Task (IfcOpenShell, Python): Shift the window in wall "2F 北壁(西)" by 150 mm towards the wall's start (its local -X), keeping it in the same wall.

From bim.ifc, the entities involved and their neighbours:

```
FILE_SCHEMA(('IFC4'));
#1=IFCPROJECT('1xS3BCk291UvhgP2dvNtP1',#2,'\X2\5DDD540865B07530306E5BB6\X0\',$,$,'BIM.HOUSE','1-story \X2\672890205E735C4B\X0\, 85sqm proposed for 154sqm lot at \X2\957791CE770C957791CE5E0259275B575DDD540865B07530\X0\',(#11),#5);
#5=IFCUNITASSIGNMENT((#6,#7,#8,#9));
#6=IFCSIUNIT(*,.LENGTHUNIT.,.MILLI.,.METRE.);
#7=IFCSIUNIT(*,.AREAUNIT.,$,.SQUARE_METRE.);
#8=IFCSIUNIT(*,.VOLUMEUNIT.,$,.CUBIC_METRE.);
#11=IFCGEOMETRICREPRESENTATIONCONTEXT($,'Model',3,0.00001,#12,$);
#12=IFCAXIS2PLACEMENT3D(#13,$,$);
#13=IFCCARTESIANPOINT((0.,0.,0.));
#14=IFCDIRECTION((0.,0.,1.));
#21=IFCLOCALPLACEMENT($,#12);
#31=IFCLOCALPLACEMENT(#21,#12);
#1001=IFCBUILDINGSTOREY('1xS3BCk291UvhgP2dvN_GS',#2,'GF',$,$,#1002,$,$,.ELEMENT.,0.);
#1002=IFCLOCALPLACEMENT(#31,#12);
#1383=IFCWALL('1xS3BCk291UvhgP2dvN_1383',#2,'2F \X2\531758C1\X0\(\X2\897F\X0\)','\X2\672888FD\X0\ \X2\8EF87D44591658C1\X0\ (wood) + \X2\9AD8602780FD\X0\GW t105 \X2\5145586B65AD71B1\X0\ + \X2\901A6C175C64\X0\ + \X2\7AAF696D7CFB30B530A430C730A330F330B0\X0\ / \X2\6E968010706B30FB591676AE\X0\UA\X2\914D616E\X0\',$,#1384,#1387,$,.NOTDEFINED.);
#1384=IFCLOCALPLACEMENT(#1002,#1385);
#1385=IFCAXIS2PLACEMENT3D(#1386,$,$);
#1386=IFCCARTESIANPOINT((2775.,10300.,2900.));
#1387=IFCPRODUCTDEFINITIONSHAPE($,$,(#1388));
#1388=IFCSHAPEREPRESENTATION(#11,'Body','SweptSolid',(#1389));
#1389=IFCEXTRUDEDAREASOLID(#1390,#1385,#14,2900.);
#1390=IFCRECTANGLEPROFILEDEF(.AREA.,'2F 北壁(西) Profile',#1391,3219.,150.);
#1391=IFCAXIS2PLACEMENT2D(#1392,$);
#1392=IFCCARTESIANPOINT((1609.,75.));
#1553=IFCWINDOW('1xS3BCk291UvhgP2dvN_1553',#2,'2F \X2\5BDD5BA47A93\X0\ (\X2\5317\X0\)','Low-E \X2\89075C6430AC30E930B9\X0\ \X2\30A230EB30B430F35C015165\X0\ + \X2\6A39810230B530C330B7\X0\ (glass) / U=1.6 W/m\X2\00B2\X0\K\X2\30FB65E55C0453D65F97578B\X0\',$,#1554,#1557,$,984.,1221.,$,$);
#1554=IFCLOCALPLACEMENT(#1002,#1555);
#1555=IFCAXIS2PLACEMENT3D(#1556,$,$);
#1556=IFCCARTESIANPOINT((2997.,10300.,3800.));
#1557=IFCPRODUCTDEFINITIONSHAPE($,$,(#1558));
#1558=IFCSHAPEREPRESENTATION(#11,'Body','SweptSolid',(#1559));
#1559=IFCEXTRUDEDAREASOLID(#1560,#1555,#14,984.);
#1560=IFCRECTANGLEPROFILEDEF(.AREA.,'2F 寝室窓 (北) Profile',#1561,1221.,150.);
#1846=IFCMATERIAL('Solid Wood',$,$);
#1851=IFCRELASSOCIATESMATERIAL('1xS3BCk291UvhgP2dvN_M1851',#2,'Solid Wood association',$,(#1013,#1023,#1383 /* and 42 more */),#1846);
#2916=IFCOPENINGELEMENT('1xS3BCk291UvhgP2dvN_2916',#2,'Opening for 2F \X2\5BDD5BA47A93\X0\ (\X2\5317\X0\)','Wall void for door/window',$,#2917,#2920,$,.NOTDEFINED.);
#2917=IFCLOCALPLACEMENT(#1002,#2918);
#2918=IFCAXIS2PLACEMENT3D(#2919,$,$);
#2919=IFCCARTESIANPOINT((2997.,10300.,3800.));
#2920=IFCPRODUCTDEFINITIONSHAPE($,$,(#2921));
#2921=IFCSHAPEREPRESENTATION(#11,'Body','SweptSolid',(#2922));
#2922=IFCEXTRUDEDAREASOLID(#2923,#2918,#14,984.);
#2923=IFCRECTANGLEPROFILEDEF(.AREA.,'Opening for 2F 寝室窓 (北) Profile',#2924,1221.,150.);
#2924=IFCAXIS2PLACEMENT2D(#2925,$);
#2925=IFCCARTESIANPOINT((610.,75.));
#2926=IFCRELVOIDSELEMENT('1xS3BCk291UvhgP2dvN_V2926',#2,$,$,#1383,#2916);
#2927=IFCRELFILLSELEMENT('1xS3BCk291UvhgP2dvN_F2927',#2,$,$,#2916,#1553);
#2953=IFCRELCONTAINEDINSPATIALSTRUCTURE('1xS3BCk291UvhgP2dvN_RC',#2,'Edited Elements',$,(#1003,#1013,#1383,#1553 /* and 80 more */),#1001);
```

```python
import ifcopenshell
import ifcopenshell.api.geometry
import ifcopenshell.util.placement
import ifcopenshell.util.unit

model = ifcopenshell.open("bim.ifc")
unit_scale = ifcopenshell.util.unit.calculate_unit_scale(model)

window = model.by_guid("1xS3BCk291UvhgP2dvN_1553")
opening = window.FillsVoids[0].RelatingOpeningElement
wall = opening.VoidsElements[0].RelatingBuildingElement

wall_matrix = ifcopenshell.util.placement.get_local_placement(wall.ObjectPlacement)
shift = wall_matrix[:3, 0] * -0.15 / unit_scale
before = ifcopenshell.util.placement.get_local_placement(window.ObjectPlacement)[:3, 3].copy()

# The window is not placed relative to its opening, so move both.
for product in (opening, window):
    matrix = ifcopenshell.util.placement.get_local_placement(product.ObjectPlacement)
    matrix[:3, 3] += shift
    ifcopenshell.api.geometry.edit_object_placement(model, product=product, matrix=matrix, is_si=False)

after = ifcopenshell.util.placement.get_local_placement(window.ObjectPlacement)[:3, 3]
print("window moved by", (after - before).round(3) + 0.0)

model.write("bim_v2.ifc")
```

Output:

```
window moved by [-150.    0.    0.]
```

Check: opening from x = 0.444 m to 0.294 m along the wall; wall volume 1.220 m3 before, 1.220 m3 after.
